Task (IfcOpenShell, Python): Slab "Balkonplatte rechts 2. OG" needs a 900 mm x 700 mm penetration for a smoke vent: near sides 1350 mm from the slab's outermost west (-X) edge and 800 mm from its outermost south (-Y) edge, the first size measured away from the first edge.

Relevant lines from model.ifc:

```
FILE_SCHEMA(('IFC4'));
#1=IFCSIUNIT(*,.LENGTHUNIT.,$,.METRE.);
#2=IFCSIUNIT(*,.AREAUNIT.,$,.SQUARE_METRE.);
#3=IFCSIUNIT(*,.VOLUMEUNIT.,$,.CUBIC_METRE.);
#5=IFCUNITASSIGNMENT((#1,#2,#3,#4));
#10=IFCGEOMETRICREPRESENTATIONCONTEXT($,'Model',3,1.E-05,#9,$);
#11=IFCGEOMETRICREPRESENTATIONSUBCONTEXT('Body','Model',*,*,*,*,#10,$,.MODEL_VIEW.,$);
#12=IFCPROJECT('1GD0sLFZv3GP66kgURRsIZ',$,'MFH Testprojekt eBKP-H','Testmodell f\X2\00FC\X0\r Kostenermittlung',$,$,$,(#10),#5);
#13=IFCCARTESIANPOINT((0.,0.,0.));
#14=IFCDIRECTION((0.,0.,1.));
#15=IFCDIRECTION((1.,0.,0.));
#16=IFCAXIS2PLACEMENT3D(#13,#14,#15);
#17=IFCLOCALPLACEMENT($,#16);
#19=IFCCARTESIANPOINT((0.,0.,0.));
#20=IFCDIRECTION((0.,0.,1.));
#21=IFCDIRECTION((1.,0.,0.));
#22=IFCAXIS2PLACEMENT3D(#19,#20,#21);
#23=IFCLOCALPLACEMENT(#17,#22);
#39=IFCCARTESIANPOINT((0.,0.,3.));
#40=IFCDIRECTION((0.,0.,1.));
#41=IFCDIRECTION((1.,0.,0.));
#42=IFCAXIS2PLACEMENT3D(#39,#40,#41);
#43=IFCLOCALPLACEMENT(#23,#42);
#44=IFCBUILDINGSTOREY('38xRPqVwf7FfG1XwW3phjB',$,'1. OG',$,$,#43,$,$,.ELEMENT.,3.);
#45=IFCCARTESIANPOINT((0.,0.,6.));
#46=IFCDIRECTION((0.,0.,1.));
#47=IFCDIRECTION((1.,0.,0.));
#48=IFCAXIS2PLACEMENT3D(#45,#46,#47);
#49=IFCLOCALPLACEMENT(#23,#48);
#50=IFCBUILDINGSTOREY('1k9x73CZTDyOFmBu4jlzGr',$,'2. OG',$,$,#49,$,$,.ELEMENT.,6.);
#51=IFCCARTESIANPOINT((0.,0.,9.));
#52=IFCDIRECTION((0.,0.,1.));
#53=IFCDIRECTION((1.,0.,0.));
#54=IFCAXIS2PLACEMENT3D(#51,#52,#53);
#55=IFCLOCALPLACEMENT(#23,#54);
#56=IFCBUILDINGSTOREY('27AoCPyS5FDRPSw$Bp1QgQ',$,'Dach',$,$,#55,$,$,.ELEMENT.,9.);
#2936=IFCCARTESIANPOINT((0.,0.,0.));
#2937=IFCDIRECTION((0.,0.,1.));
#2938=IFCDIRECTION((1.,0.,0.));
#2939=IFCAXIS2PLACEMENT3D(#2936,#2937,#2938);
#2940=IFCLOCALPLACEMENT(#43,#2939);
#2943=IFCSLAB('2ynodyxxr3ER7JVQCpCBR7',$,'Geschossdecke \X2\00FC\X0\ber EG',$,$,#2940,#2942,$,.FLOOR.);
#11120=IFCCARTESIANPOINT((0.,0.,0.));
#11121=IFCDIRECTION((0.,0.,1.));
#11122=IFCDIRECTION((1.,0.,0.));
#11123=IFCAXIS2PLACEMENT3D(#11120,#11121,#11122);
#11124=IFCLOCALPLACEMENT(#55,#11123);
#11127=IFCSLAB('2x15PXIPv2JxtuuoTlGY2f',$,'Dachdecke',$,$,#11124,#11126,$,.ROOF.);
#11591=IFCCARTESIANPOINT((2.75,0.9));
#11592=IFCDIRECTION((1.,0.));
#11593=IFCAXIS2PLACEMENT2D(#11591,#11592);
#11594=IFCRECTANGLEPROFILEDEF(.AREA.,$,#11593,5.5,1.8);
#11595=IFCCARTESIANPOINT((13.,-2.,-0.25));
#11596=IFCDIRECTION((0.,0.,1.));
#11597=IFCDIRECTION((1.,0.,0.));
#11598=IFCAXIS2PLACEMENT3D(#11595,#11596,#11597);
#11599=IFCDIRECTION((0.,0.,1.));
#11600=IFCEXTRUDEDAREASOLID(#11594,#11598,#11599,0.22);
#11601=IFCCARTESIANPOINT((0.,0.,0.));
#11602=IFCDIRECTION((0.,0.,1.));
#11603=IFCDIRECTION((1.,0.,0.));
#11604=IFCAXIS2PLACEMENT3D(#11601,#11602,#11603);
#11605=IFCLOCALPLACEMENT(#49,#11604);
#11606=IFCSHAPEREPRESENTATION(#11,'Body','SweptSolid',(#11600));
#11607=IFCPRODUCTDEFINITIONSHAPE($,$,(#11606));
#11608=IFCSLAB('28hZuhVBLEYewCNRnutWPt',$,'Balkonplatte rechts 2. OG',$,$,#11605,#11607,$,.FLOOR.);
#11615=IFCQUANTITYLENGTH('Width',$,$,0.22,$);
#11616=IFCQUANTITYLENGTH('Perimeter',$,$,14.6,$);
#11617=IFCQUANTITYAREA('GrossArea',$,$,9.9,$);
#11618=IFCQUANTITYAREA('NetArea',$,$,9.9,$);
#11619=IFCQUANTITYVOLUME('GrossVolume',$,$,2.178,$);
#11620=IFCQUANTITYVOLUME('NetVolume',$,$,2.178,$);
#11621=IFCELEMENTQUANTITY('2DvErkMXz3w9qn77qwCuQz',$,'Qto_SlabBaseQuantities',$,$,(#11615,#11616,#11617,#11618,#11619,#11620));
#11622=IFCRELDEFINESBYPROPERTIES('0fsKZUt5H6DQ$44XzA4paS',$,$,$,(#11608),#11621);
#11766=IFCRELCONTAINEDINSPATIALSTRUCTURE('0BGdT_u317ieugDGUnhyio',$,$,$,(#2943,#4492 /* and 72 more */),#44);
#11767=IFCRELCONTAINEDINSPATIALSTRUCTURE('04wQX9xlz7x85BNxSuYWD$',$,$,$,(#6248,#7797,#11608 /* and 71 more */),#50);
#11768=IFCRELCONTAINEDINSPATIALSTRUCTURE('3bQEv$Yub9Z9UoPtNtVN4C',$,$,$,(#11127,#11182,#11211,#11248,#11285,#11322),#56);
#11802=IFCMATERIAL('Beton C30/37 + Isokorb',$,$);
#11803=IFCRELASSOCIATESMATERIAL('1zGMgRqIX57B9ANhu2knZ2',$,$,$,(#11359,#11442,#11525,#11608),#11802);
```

```python
import numpy as np
import ifcopenshell
import ifcopenshell.api.feature
import ifcopenshell.api.geometry
import ifcopenshell.api.pset
import ifcopenshell.api.root
import ifcopenshell.geom
import ifcopenshell.util.element
import ifcopenshell.util.placement
import ifcopenshell.util.representation
import ifcopenshell.util.shape
import ifcopenshell.util.unit

model = ifcopenshell.open("model.ifc")
unit_scale = ifcopenshell.util.unit.calculate_unit_scale(model)
area_scale = ifcopenshell.util.unit.calculate_unit_scale(model, "AREAUNIT")
volume_scale = ifcopenshell.util.unit.calculate_unit_scale(model, "VOLUMEUNIT")
settings = ifcopenshell.geom.settings()


def volume(element):
    """Net volume in cubic metres, openings subtracted."""
    shape = ifcopenshell.geom.create_shape(settings, element)
    return ifcopenshell.util.shape.get_volume(shape.geometry)


slab = model.by_guid("28hZuhVBLEYewCNRnutWPt")
before = volume(slab)

# Extent in the slab's own axes, in metres. The edges named are its -X and -Y sides.
slab_shape = ifcopenshell.geom.create_shape(settings, slab)
vertices = ifcopenshell.util.shape.get_vertices(slab_shape.geometry)
x_min, y_min, bottom = vertices.min(axis=0)
top = vertices[:, 2].max()

opening = ifcopenshell.api.root.create_entity(model, ifc_class="IfcOpeningElement", name="Smoke vent opening", predefined_type="OPENING")
context = ifcopenshell.util.representation.get_context(model, "Model", "Body", "MODEL_VIEW")
width, depth = 0.9, 0.7
outline = [(0.0, 0.0), (width, 0.0), (width, depth), (0.0, depth), (0.0, 0.0)]
# Overshoot both faces by 50 mm so the cut is clean.
shape = ifcopenshell.api.geometry.add_slab_representation(
    model, context=context, depth=top - bottom + 0.1, polyline=outline
)
ifcopenshell.api.geometry.assign_representation(model, product=opening, representation=shape)

matrix = ifcopenshell.util.placement.get_local_placement(slab.ObjectPlacement)
matrix[:, 3] = matrix @ np.append(np.array([x_min + 1.35, y_min + 0.8, bottom - 0.05]) / unit_scale, 1.0)
ifcopenshell.api.geometry.edit_object_placement(model, product=opening, matrix=matrix, is_si=False)
ifcopenshell.api.feature.add_feature(model, feature=opening, element=slab)

after = volume(slab)

# Update the slab's stored quantities.
qto = model.by_id(ifcopenshell.util.element.get_pset(slab, "Qto_SlabBaseQuantities", should_inherit=False)["id"])
ifcopenshell.api.pset.edit_qto(model, qto=qto, properties={
    "NetArea": after / (top - bottom) / area_scale,
    "NetVolume": after / volume_scale,
})

print(f"slab volume {before:.3f} -> {after:.3f} m3")

model.write("model_v2.ifc")
```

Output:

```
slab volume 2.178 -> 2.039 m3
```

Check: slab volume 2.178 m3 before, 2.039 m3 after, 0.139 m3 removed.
